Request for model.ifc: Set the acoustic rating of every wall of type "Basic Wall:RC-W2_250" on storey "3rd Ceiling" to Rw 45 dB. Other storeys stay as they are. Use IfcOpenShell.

First a look at what the model holds.

```python
import ifcopenshell
import ifcopenshell.util.element

model = ifcopenshell.open("model.ifc")
print(model.schema)
storey = next(s for s in model.by_type("IfcBuildingStorey") if s.Name == "3rd Ceiling")
walls = [e for e in ifcopenshell.util.element.get_decomposition(storey) if e.is_a("IfcWall")]
seen = {}
for e in walls:
    element_type = ifcopenshell.util.element.get_type(e)
    key = (element_type.Name if element_type != e and element_type else None, ifcopenshell.util.element.get_pset(e, "Pset_WallCommon", "AcousticRating"))
    seen[key] = seen.get(key, 0) + 1
for (name, value), count in sorted(seen.items(), key=str):
    print(count, "x", name, "|", value)
```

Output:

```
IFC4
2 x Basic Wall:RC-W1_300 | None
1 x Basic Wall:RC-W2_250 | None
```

```python
import ifcopenshell
import ifcopenshell.api.pset
import ifcopenshell.util.element

model = ifcopenshell.open("model.ifc")

storey = next(s for s in model.by_type("IfcBuildingStorey") if s.Name == "3rd Ceiling")
walls = [e for e in ifcopenshell.util.element.get_decomposition(storey) if e.is_a("IfcWall")]

count = 0
for e in walls:
    element_type = ifcopenshell.util.element.get_type(e)
    if element_type in (None, e) or element_type.Name != "Basic Wall:RC-W2_250":
        continue
    # add_pset returns the element's existing set when there is one.
    pset = ifcopenshell.api.pset.add_pset(model, product=e, name="Pset_WallCommon")
    ifcopenshell.api.pset.edit_pset(model, pset=pset, properties={"AcousticRating": "Rw 45 dB"})
    count += 1

print(count, "walls updated")

model.write("model-out.ifc")
```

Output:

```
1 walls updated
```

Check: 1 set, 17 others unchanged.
